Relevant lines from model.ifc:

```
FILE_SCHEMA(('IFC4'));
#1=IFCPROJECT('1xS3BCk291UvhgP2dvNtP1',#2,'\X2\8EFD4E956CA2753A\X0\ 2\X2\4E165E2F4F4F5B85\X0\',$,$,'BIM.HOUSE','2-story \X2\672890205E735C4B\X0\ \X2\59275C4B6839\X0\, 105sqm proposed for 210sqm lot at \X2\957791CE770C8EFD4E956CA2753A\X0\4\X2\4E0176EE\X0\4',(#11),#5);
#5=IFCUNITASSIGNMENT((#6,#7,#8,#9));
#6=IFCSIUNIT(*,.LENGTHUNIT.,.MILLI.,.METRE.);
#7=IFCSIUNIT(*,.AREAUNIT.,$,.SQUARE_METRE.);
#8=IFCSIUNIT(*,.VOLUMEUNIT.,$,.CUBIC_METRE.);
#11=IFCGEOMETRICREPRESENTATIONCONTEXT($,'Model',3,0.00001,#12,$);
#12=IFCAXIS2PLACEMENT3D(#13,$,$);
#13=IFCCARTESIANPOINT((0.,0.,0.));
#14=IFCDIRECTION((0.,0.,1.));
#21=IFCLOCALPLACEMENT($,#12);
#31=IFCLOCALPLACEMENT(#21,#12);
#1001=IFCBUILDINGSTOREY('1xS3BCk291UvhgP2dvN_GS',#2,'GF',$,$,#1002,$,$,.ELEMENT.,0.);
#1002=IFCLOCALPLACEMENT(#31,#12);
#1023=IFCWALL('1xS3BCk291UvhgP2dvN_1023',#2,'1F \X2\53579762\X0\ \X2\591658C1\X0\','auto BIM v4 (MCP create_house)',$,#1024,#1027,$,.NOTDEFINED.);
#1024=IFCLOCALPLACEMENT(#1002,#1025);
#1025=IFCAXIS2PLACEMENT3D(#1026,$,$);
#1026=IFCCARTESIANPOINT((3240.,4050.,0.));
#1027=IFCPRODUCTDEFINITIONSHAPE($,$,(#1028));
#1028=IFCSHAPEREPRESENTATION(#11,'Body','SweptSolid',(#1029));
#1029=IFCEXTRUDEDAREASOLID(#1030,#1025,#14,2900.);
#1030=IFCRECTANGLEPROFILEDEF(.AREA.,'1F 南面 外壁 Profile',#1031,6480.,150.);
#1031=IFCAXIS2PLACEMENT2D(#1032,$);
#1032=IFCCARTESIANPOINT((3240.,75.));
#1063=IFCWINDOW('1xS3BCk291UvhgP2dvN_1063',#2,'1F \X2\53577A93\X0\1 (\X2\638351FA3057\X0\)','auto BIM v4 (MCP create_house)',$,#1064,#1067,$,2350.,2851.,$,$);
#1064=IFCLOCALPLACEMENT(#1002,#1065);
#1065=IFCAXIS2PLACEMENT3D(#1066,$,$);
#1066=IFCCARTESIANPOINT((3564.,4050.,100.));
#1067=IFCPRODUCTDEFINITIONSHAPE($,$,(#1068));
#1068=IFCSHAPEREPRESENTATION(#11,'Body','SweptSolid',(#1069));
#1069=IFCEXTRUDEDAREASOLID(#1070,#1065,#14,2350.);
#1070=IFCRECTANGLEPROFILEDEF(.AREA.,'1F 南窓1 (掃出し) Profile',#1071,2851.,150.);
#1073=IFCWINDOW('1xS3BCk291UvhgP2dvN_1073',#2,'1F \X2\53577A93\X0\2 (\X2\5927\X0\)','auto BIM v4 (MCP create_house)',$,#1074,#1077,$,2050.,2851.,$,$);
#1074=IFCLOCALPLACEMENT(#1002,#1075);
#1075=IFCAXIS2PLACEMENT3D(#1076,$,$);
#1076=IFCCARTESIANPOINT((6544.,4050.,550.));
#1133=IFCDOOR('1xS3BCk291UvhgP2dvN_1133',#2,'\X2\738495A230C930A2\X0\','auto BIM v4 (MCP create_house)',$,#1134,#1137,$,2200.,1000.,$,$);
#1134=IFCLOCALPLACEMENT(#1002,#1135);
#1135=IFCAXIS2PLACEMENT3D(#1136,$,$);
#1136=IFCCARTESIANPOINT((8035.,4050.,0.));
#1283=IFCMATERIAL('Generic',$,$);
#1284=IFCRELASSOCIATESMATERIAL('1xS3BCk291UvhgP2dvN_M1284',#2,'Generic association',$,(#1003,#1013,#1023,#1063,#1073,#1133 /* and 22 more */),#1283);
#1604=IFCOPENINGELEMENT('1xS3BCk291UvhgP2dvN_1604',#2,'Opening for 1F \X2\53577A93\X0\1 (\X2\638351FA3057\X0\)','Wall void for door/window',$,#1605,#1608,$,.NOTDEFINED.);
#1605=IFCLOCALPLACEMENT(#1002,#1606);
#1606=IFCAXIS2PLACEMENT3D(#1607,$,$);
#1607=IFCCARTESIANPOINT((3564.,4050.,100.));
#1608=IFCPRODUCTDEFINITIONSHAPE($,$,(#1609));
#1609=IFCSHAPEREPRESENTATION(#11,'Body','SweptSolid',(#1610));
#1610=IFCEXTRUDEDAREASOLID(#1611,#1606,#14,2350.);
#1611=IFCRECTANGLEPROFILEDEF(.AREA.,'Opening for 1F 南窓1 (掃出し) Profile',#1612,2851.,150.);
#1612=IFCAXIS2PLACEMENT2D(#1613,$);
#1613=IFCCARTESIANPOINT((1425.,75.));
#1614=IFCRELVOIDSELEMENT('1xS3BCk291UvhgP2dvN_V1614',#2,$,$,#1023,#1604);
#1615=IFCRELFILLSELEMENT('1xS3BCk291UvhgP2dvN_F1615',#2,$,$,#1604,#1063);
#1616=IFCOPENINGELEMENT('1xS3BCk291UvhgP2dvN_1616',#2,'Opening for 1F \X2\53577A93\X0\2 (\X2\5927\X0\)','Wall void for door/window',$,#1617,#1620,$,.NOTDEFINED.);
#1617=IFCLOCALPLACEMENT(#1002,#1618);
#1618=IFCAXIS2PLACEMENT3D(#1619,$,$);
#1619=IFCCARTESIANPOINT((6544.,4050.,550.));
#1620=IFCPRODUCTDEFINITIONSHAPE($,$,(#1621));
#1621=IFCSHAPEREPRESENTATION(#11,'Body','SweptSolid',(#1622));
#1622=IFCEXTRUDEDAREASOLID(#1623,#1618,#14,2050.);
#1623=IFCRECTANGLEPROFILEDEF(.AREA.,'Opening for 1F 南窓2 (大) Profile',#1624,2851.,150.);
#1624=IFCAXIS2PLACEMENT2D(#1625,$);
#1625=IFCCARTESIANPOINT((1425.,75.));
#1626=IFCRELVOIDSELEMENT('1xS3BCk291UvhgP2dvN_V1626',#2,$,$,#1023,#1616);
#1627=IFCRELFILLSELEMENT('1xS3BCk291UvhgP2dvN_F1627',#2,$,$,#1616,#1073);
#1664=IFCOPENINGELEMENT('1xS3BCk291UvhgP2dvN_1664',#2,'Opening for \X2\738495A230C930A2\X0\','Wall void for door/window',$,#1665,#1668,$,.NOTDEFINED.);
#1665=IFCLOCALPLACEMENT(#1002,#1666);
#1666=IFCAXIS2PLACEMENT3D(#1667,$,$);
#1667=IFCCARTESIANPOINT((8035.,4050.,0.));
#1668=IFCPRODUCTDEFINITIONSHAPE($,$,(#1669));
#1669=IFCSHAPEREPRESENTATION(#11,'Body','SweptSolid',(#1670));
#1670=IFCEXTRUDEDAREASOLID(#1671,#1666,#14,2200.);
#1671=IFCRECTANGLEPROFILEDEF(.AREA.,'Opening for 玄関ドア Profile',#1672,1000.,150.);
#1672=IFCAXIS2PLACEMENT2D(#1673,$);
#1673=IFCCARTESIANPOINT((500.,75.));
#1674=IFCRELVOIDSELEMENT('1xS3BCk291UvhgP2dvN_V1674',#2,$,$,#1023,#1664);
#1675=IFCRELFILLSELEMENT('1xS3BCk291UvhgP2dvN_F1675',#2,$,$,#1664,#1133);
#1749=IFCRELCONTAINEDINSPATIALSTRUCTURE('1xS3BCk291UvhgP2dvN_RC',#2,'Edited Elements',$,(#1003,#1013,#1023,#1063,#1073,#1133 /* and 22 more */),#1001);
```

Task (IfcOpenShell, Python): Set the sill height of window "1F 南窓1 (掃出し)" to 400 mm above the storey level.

```python
import numpy as np
import ifcopenshell
import ifcopenshell.api.geometry
import ifcopenshell.geom
import ifcopenshell.util.element
import ifcopenshell.util.placement
import ifcopenshell.util.shape
import ifcopenshell.util.unit

model = ifcopenshell.open("model.ifc")
unit_scale = ifcopenshell.util.unit.calculate_unit_scale(model)

window = model.by_guid("1xS3BCk291UvhgP2dvN_1063")
opening = window.FillsVoids[0].RelatingOpeningElement
storey = ifcopenshell.util.element.get_container(window, ifc_class="IfcBuildingStorey")
level = ifcopenshell.util.placement.get_local_placement(storey.ObjectPlacement)[2, 3]

# The opening's origin need not be at the sill, so measure its lowest point.
shape = ifcopenshell.geom.create_shape(ifcopenshell.geom.settings(), opening)
bottom = ifcopenshell.util.shape.get_shape_bottom_elevation(shape, shape.geometry) / unit_scale
dz = level + 400.0 - bottom

shift = np.array([0.0, 0.0, dz])
# The window is not placed relative to its opening, so move both.
for product in (opening, window):
    matrix = ifcopenshell.util.placement.get_local_placement(product.ObjectPlacement)
    matrix[:3, 3] += shift
    ifcopenshell.api.geometry.edit_object_placement(model, product=product, matrix=matrix, is_si=False)

print(f"moved by {dz * unit_scale:+.3f} m")

model.write("model-out.ifc")
```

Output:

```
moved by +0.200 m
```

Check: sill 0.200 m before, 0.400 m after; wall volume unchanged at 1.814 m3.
